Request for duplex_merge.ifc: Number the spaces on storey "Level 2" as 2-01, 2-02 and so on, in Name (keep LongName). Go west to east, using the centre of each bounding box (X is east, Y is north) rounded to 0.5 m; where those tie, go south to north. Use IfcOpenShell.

First a look at what the model holds.

```python
import ifcopenshell
import ifcopenshell.util.element
import ifcopenshell.util.placement

model = ifcopenshell.open("duplex_merge.ifc")
print(model.schema)
storey = next(s for s in model.by_type("IfcBuildingStorey") if s.Name == "Level 2")
spaces = [e for e in ifcopenshell.util.element.get_decomposition(storey) if e.is_a("IfcSpace")]
for e in sorted(spaces, key=lambda e: e.id()):
    origin = ifcopenshell.util.placement.get_local_placement(e.ObjectPlacement)[:3, 3]
    print(e.id(), e.Name, e.LongName, origin.round(2) + 0.0, sep=" | ")
```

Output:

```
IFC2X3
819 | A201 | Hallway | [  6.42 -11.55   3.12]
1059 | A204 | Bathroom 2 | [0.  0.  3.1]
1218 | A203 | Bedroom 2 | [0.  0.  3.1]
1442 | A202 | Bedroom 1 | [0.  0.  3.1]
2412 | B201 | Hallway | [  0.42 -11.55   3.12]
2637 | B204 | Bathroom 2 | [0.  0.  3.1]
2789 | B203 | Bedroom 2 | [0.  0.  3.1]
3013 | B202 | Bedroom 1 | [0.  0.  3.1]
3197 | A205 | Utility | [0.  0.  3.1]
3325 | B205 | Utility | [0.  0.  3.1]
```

```python
import ifcopenshell
import ifcopenshell.geom
import ifcopenshell.util.element
import ifcopenshell.util.shape

model = ifcopenshell.open("duplex_merge.ifc")
settings = ifcopenshell.geom.settings()
settings.set("use-world-coords", True)


def centre(element):
    shape = ifcopenshell.geom.create_shape(settings, element)
    return ifcopenshell.util.shape.get_bbox_centroid(shape.geometry)


storey = next(s for s in model.by_type("IfcBuildingStorey") if s.Name == "Level 2")
spaces = [e for e in ifcopenshell.util.element.get_decomposition(storey) if e.is_a("IfcSpace")]

# Insertion points can sit at a corner or the storey origin, so sort by the geometry (in metres).
centres = {e: centre(e) for e in spaces}
spaces.sort(key=lambda e: (round(centres[e][0] / 0.5), centres[e][1]))

for i, e in enumerate(spaces, start=1):
    number = f"2-{i:02d}"
    e.Name = number
    print(e.id(), number)

model.write("duplex_merge-out.ifc")
```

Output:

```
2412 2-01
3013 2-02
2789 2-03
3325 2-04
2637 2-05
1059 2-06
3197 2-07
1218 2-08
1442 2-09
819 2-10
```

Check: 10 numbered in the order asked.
